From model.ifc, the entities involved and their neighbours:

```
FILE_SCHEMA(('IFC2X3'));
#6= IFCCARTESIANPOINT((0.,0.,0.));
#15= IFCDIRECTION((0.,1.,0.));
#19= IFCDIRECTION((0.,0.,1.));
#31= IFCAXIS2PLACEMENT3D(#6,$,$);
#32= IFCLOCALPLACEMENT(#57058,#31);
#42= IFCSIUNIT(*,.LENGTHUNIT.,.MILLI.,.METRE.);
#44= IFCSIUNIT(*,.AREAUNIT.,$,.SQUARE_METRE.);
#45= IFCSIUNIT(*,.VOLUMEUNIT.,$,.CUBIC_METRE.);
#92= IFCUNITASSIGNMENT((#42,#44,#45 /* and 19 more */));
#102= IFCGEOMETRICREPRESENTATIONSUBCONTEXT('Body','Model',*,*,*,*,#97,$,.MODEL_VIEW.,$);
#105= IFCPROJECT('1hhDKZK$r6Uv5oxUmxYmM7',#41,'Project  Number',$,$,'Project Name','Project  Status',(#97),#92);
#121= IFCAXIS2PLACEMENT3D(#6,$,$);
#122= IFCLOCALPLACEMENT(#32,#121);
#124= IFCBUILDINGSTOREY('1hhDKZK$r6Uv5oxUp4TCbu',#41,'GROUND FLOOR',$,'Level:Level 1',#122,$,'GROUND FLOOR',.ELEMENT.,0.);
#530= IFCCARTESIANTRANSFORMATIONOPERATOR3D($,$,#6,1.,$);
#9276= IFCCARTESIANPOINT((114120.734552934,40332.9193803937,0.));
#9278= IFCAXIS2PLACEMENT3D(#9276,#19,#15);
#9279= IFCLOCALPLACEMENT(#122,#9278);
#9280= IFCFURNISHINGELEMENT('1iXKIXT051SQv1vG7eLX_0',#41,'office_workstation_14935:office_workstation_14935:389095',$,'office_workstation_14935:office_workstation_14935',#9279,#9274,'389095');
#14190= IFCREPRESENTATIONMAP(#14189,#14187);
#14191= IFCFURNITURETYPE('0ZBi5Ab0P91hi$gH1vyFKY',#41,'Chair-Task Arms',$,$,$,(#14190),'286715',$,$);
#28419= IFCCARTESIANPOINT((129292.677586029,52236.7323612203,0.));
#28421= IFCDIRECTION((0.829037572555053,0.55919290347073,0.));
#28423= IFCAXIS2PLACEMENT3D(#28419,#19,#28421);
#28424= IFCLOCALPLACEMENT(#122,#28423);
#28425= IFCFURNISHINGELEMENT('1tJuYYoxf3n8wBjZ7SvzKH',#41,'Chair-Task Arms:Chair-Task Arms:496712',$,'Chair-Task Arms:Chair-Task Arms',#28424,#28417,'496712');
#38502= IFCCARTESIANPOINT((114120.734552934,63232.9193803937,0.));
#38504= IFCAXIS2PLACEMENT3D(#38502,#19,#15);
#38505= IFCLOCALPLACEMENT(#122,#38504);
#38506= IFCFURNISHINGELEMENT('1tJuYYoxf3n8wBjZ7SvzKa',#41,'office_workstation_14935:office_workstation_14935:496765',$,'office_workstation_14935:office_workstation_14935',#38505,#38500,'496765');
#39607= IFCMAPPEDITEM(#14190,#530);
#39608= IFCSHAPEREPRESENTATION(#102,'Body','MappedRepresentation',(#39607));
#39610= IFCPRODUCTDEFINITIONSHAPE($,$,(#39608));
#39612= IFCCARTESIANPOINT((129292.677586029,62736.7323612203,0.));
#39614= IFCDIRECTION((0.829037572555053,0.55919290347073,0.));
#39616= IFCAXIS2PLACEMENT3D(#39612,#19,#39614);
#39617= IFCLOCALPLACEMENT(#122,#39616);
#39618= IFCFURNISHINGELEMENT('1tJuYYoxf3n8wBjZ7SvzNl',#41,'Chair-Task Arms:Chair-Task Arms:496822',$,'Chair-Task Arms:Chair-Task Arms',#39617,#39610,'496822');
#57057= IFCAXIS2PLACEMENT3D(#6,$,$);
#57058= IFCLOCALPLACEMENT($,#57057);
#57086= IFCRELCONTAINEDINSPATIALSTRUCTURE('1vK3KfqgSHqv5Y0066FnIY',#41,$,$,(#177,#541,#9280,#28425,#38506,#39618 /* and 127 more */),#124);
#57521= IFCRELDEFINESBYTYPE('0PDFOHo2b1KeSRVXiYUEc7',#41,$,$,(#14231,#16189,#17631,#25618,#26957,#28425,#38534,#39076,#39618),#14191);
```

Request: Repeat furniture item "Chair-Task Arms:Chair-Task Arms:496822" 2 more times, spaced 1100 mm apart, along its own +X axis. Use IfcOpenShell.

```python
import ifcopenshell
import ifcopenshell.api.geometry
import ifcopenshell.api.root
import ifcopenshell.util.element
import ifcopenshell.util.placement
import ifcopenshell.util.unit

model = ifcopenshell.open("model.ifc")
unit_scale = ifcopenshell.util.unit.calculate_unit_scale(model)


def reuse_history(source, copy):
    """copy_class also copies each property set's owner history, people and application; keep the originals."""
    for rel in copy.IsDefinedBy:
        if rel.is_a("IfcRelDefinesByProperties") and (history := rel.RelatingPropertyDefinition.OwnerHistory):
            rel.RelatingPropertyDefinition.OwnerHistory = source.OwnerHistory
            ifcopenshell.util.element.remove_deep2(model, history)


source = model.by_id(39618)
base = ifcopenshell.util.placement.get_local_placement(source.ObjectPlacement)
step = base[:3, 0] * 1.1 / unit_scale

for i in range(1, 3):
    copy = ifcopenshell.api.root.copy_class(model, product=source)
    copy.Representation = ifcopenshell.util.element.copy_deep(
        model, source.Representation, exclude=["IfcGeometricRepresentationContext", "IfcRepresentationMap"]
    )
    copy.Name = "Chair-Task Arms:Chair-Task Arms"
    copy.Tag = None
    reuse_history(source, copy)
    matrix = base.copy()
    matrix[:3, 3] += i * step
    print("added at", matrix[:3, 3].round(3) + 0.0)
    ifcopenshell.api.geometry.edit_object_placement(model, product=copy, matrix=matrix, is_si=False)

model.write("model_updated.ifc")
```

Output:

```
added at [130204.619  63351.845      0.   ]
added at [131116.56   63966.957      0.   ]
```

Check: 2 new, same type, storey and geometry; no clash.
